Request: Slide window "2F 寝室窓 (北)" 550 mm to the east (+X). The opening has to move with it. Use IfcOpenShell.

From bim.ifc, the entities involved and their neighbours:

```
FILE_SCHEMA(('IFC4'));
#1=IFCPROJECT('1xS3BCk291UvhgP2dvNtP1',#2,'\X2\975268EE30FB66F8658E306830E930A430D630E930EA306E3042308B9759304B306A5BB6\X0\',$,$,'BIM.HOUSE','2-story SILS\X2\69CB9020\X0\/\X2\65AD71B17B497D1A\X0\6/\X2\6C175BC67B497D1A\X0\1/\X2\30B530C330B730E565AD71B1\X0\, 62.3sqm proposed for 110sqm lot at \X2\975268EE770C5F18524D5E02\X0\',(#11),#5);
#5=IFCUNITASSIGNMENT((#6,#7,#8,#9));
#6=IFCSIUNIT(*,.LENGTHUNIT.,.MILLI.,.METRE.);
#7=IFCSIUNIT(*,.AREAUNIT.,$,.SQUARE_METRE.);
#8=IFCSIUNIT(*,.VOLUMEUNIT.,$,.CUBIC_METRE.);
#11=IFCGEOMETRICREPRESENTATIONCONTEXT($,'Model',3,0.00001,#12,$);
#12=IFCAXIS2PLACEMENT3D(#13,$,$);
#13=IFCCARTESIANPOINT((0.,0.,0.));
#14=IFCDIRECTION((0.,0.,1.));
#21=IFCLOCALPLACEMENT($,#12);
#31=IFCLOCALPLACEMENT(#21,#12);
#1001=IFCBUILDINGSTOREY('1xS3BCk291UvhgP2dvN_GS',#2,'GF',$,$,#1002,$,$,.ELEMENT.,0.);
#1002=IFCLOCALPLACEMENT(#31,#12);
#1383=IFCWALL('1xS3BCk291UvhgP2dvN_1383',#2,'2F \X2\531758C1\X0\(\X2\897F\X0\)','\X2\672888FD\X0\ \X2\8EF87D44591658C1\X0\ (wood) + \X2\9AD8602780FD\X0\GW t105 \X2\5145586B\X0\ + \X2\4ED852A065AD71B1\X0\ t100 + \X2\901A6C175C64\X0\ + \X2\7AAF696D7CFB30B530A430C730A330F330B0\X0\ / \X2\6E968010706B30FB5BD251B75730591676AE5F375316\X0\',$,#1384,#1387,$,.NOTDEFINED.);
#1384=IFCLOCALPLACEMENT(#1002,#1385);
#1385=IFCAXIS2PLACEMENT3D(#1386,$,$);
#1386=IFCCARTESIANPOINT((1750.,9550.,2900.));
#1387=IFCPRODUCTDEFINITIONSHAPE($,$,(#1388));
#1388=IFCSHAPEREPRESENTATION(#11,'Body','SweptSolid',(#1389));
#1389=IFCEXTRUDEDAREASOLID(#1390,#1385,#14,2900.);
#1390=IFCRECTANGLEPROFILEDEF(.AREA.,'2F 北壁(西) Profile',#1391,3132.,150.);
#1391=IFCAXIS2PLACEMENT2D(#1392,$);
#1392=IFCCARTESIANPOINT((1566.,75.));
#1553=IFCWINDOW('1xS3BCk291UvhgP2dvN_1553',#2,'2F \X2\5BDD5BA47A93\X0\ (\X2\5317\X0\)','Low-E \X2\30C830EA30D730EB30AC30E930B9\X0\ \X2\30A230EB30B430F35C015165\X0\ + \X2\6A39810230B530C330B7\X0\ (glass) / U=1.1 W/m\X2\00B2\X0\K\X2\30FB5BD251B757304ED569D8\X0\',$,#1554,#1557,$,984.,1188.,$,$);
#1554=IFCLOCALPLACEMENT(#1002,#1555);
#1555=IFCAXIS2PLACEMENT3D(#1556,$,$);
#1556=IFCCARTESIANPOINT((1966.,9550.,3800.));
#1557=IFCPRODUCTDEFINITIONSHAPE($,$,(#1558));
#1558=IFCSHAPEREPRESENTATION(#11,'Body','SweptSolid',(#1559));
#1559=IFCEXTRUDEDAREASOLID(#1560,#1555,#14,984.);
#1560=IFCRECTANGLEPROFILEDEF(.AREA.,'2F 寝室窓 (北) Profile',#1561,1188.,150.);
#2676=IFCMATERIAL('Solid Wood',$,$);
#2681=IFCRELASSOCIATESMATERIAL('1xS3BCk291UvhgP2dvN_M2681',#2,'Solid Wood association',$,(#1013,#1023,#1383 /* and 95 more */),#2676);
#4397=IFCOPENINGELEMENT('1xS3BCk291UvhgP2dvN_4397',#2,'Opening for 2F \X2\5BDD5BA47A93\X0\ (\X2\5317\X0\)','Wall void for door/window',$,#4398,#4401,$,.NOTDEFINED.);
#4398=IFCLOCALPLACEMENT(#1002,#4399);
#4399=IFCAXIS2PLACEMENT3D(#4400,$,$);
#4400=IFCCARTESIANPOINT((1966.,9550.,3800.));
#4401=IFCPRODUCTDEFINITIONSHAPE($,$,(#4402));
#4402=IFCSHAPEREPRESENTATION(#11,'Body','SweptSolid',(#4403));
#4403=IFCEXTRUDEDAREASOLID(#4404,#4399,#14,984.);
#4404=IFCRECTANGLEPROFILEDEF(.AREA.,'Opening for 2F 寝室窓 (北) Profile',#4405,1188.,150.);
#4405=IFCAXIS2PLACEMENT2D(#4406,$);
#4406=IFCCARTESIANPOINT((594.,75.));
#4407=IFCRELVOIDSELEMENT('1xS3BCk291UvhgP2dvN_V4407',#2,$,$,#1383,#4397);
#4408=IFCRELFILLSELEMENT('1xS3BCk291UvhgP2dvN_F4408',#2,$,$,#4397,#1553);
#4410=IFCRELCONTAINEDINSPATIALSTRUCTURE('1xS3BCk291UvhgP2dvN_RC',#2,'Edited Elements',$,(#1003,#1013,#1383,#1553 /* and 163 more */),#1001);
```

```python
import ifcopenshell
import ifcopenshell.api.geometry
import ifcopenshell.util.placement
import ifcopenshell.util.unit

model = ifcopenshell.open("bim.ifc")
unit_scale = ifcopenshell.util.unit.calculate_unit_scale(model)

window = model.by_guid("1xS3BCk291UvhgP2dvN_1553")
opening = window.FillsVoids[0].RelatingOpeningElement
wall = opening.VoidsElements[0].RelatingBuildingElement

wall_matrix = ifcopenshell.util.placement.get_local_placement(wall.ObjectPlacement)
shift = wall_matrix[:3, 0] * 0.55 / unit_scale
before = ifcopenshell.util.placement.get_local_placement(window.ObjectPlacement)[:3, 3].copy()

# The window is not placed relative to its opening, so move both.
for product in (opening, window):
    matrix = ifcopenshell.util.placement.get_local_placement(product.ObjectPlacement)
    matrix[:3, 3] += shift
    ifcopenshell.api.geometry.edit_object_placement(model, product=product, matrix=matrix, is_si=False)

after = ifcopenshell.util.placement.get_local_placement(window.ObjectPlacement)[:3, 3]
print("window moved by", (after - before).round(3) + 0.0)

model.write("bim-out.ifc")
```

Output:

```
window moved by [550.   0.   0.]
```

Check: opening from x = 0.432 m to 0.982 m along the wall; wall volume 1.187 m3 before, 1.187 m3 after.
